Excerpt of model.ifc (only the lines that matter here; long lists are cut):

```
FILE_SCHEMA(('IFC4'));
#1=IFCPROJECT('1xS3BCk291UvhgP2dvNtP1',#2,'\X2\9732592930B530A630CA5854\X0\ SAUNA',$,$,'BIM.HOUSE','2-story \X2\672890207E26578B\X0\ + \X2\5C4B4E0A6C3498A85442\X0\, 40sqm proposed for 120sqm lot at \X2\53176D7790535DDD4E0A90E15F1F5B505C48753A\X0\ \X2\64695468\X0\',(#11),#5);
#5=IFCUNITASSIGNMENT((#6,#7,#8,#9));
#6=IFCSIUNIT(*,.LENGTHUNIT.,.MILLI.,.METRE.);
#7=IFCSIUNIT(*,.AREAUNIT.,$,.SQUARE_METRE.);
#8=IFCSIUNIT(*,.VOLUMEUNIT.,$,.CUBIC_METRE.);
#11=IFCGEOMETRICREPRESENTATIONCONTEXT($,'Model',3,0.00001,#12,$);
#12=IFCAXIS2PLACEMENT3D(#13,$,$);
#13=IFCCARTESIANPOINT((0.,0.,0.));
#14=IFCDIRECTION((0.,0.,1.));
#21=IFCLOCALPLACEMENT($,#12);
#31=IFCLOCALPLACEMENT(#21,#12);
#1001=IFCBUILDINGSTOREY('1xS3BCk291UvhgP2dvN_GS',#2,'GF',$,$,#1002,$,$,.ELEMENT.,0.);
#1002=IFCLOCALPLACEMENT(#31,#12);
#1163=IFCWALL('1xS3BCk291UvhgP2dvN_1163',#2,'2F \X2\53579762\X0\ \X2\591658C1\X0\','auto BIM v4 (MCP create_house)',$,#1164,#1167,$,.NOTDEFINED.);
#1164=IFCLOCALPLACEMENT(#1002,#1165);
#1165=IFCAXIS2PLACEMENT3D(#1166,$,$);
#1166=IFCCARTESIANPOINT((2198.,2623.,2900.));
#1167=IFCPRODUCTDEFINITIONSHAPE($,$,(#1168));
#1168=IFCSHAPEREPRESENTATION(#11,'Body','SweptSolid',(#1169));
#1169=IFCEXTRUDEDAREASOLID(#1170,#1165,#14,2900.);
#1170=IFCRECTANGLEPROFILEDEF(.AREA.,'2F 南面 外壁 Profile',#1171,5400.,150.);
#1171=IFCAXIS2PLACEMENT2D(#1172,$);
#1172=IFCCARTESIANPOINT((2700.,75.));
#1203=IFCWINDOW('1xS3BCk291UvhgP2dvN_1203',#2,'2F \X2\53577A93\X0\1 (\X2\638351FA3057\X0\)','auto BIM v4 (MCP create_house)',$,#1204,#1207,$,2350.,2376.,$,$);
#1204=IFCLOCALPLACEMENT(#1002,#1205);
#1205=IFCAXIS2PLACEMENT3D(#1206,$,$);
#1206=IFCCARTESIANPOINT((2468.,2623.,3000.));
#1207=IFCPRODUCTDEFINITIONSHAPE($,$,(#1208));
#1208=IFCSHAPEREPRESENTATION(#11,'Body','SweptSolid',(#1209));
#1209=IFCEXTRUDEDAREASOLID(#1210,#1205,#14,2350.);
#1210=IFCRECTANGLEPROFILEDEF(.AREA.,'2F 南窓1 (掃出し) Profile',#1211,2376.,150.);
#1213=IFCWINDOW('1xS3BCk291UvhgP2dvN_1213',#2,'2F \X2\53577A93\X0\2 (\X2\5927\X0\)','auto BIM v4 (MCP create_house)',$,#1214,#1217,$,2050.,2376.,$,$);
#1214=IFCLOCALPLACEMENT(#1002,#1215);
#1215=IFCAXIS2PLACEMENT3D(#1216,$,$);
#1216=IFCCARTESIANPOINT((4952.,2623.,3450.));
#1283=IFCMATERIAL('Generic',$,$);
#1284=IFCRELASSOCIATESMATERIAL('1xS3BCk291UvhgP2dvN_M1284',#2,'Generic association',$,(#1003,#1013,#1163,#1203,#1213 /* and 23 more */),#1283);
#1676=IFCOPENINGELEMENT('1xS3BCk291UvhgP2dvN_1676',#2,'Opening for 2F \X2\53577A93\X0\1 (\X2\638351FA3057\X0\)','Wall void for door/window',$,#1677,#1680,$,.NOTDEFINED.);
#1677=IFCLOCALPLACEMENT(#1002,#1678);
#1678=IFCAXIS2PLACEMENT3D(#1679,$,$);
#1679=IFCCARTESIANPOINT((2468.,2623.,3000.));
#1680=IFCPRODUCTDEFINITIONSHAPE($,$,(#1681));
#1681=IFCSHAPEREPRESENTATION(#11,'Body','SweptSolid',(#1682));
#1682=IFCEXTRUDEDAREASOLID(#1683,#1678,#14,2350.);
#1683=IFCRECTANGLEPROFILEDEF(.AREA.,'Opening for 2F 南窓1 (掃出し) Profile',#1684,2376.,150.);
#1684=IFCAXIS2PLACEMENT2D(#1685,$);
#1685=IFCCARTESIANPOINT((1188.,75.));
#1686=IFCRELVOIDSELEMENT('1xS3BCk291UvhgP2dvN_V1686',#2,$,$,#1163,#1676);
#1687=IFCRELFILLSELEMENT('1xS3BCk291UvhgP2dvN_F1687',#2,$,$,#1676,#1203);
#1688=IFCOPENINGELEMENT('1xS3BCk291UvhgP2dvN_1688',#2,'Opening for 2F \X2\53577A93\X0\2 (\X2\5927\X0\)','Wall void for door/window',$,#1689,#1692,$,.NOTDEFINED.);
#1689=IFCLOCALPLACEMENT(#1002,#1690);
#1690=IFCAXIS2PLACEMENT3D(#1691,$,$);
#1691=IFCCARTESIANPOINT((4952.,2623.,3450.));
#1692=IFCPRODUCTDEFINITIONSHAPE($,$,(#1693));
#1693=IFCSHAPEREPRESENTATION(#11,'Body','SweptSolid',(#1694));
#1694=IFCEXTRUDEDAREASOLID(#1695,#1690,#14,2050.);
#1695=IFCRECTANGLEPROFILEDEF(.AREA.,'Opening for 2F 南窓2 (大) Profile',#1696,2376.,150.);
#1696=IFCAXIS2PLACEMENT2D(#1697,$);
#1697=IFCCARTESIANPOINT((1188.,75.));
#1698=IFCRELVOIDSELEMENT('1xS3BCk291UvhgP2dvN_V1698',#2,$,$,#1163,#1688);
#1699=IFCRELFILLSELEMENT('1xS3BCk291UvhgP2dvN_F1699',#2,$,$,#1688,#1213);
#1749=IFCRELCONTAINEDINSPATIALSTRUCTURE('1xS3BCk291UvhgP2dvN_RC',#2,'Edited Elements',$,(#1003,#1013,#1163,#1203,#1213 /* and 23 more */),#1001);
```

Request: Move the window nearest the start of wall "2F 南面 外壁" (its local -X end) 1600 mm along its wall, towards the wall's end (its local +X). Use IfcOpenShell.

```python
import ifcopenshell
import ifcopenshell.api.geometry
import ifcopenshell.util.placement
import ifcopenshell.util.unit

model = ifcopenshell.open("model.ifc")
unit_scale = ifcopenshell.util.unit.calculate_unit_scale(model)

window = model.by_guid("1xS3BCk291UvhgP2dvN_1203")
opening = window.FillsVoids[0].RelatingOpeningElement
wall = opening.VoidsElements[0].RelatingBuildingElement

wall_matrix = ifcopenshell.util.placement.get_local_placement(wall.ObjectPlacement)
shift = wall_matrix[:3, 0] * 1.6 / unit_scale
before = ifcopenshell.util.placement.get_local_placement(window.ObjectPlacement)[:3, 3].copy()

# The window is not placed relative to its opening, so move both.
for product in (opening, window):
    matrix = ifcopenshell.util.placement.get_local_placement(product.ObjectPlacement)
    matrix[:3, 3] += shift
    ifcopenshell.api.geometry.edit_object_placement(model, product=product, matrix=matrix, is_si=False)

after = ifcopenshell.util.placement.get_local_placement(window.ObjectPlacement)[:3, 3]
print("window moved by", (after - before).round(3) + 0.0)

model.write("model_edited.ifc")
```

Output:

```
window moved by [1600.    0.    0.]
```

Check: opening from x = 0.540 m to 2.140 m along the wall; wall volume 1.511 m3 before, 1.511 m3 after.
